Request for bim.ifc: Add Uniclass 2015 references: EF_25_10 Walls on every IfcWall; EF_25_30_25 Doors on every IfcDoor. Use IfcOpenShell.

First a look at what the model holds.

```python
import ifcopenshell

model = ifcopenshell.open("bim.ifc")
print(model.schema)
print("classifications:", [c.Name for c in model.by_type("IfcClassification")])
for ifc_class in ("IfcDoor", "IfcRoof", "IfcStair", "IfcWall", "IfcWindow"):
    print(ifc_class, len(model.by_type(ifc_class)))
```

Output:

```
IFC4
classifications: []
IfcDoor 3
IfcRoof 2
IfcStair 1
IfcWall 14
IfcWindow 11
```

```python
import ifcopenshell
import ifcopenshell.api.classification

model = ifcopenshell.open("bim.ifc")

system = ifcopenshell.api.classification.add_classification(model, classification="Uniclass 2015")

codes = {
    "IfcWall": ("EF_25_10", "Walls"),
    "IfcDoor": ("EF_25_30_25", "Doors"),
}
for ifc_class, (code, name) in codes.items():
    products = model.by_type(ifc_class)
    ifcopenshell.api.classification.add_reference(
        model, products=products, classification=system, identification=code, name=name
    )
    print(code, len(products))

model.write("bim_rev.ifc")
```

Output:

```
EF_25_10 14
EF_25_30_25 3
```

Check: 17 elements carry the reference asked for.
